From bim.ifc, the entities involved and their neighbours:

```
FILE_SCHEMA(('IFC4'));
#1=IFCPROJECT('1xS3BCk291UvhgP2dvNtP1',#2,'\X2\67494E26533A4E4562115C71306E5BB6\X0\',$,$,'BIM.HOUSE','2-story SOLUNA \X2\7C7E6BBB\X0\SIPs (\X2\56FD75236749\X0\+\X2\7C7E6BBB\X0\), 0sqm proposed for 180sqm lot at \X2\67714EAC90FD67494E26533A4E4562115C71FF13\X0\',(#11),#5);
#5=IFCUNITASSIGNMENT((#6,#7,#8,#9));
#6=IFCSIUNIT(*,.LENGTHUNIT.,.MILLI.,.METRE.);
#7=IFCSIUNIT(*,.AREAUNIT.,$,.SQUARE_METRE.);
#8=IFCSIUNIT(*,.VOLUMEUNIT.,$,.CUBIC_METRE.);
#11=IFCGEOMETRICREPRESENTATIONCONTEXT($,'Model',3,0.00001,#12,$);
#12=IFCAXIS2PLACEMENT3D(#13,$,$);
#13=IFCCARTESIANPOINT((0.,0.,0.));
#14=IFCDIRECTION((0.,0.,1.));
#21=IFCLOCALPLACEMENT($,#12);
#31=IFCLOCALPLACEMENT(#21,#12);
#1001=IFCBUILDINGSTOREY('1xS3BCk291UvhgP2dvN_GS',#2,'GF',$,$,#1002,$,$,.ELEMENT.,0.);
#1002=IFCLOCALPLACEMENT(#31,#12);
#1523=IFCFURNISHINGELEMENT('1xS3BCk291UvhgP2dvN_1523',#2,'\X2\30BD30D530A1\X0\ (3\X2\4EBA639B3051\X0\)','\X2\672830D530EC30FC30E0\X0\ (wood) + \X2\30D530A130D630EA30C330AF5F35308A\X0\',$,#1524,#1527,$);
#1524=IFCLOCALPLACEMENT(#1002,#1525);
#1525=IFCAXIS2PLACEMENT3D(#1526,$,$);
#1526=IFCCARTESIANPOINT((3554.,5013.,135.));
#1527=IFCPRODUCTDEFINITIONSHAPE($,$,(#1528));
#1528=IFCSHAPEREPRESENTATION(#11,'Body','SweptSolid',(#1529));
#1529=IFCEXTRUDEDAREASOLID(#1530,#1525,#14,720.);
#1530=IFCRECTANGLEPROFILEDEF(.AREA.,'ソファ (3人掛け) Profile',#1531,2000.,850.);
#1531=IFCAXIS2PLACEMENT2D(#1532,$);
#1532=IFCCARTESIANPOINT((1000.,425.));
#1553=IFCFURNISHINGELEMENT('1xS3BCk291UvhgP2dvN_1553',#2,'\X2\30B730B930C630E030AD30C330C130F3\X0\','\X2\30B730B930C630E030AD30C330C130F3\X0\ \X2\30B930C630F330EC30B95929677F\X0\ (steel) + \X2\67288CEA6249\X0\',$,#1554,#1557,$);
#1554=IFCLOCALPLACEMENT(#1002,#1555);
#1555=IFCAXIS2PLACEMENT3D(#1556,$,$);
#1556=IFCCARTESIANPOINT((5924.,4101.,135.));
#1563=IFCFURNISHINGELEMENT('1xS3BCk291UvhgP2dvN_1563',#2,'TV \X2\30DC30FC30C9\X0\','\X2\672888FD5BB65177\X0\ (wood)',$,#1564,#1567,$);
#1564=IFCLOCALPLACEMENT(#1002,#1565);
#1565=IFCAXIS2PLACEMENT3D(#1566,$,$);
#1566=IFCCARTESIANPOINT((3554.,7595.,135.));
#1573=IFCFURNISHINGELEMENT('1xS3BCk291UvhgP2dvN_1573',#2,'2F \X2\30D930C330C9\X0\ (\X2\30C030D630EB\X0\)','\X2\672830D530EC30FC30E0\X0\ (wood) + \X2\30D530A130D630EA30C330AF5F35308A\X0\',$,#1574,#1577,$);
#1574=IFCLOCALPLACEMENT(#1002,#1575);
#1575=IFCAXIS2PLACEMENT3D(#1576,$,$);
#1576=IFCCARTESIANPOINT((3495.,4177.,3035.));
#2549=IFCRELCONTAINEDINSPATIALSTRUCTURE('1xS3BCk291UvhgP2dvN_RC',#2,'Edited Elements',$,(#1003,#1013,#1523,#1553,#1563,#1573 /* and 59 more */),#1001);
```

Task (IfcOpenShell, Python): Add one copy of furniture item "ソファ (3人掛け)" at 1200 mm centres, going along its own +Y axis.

```python
import ifcopenshell
import ifcopenshell.api.geometry
import ifcopenshell.api.root
import ifcopenshell.util.element
import ifcopenshell.util.placement

model = ifcopenshell.open("bim.ifc")


def reuse_history(source, copy):
    """copy_class also copies each property set's owner history, people and application; keep the originals."""
    for rel in copy.IsDefinedBy:
        if rel.is_a("IfcRelDefinesByProperties") and (history := rel.RelatingPropertyDefinition.OwnerHistory):
            rel.RelatingPropertyDefinition.OwnerHistory = source.OwnerHistory
            ifcopenshell.util.element.remove_deep2(model, history)


source = model.by_guid("1xS3BCk291UvhgP2dvN_1523")
base = ifcopenshell.util.placement.get_local_placement(source.ObjectPlacement)
step = base[:3, 1] * 1200.0

for i in range(1, 2):
    copy = ifcopenshell.api.root.copy_class(model, product=source)
    copy.Representation = ifcopenshell.util.element.copy_deep(
        model, source.Representation, exclude=["IfcGeometricRepresentationContext", "IfcRepresentationMap"]
    )
    reuse_history(source, copy)
    matrix = base.copy()
    matrix[:3, 3] += i * step
    print("added at", matrix[:3, 3].round(3) + 0.0)
    ifcopenshell.api.geometry.edit_object_placement(model, product=copy, matrix=matrix, is_si=False)

model.write("bim_updated.ifc")
```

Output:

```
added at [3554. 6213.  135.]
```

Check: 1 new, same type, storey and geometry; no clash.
